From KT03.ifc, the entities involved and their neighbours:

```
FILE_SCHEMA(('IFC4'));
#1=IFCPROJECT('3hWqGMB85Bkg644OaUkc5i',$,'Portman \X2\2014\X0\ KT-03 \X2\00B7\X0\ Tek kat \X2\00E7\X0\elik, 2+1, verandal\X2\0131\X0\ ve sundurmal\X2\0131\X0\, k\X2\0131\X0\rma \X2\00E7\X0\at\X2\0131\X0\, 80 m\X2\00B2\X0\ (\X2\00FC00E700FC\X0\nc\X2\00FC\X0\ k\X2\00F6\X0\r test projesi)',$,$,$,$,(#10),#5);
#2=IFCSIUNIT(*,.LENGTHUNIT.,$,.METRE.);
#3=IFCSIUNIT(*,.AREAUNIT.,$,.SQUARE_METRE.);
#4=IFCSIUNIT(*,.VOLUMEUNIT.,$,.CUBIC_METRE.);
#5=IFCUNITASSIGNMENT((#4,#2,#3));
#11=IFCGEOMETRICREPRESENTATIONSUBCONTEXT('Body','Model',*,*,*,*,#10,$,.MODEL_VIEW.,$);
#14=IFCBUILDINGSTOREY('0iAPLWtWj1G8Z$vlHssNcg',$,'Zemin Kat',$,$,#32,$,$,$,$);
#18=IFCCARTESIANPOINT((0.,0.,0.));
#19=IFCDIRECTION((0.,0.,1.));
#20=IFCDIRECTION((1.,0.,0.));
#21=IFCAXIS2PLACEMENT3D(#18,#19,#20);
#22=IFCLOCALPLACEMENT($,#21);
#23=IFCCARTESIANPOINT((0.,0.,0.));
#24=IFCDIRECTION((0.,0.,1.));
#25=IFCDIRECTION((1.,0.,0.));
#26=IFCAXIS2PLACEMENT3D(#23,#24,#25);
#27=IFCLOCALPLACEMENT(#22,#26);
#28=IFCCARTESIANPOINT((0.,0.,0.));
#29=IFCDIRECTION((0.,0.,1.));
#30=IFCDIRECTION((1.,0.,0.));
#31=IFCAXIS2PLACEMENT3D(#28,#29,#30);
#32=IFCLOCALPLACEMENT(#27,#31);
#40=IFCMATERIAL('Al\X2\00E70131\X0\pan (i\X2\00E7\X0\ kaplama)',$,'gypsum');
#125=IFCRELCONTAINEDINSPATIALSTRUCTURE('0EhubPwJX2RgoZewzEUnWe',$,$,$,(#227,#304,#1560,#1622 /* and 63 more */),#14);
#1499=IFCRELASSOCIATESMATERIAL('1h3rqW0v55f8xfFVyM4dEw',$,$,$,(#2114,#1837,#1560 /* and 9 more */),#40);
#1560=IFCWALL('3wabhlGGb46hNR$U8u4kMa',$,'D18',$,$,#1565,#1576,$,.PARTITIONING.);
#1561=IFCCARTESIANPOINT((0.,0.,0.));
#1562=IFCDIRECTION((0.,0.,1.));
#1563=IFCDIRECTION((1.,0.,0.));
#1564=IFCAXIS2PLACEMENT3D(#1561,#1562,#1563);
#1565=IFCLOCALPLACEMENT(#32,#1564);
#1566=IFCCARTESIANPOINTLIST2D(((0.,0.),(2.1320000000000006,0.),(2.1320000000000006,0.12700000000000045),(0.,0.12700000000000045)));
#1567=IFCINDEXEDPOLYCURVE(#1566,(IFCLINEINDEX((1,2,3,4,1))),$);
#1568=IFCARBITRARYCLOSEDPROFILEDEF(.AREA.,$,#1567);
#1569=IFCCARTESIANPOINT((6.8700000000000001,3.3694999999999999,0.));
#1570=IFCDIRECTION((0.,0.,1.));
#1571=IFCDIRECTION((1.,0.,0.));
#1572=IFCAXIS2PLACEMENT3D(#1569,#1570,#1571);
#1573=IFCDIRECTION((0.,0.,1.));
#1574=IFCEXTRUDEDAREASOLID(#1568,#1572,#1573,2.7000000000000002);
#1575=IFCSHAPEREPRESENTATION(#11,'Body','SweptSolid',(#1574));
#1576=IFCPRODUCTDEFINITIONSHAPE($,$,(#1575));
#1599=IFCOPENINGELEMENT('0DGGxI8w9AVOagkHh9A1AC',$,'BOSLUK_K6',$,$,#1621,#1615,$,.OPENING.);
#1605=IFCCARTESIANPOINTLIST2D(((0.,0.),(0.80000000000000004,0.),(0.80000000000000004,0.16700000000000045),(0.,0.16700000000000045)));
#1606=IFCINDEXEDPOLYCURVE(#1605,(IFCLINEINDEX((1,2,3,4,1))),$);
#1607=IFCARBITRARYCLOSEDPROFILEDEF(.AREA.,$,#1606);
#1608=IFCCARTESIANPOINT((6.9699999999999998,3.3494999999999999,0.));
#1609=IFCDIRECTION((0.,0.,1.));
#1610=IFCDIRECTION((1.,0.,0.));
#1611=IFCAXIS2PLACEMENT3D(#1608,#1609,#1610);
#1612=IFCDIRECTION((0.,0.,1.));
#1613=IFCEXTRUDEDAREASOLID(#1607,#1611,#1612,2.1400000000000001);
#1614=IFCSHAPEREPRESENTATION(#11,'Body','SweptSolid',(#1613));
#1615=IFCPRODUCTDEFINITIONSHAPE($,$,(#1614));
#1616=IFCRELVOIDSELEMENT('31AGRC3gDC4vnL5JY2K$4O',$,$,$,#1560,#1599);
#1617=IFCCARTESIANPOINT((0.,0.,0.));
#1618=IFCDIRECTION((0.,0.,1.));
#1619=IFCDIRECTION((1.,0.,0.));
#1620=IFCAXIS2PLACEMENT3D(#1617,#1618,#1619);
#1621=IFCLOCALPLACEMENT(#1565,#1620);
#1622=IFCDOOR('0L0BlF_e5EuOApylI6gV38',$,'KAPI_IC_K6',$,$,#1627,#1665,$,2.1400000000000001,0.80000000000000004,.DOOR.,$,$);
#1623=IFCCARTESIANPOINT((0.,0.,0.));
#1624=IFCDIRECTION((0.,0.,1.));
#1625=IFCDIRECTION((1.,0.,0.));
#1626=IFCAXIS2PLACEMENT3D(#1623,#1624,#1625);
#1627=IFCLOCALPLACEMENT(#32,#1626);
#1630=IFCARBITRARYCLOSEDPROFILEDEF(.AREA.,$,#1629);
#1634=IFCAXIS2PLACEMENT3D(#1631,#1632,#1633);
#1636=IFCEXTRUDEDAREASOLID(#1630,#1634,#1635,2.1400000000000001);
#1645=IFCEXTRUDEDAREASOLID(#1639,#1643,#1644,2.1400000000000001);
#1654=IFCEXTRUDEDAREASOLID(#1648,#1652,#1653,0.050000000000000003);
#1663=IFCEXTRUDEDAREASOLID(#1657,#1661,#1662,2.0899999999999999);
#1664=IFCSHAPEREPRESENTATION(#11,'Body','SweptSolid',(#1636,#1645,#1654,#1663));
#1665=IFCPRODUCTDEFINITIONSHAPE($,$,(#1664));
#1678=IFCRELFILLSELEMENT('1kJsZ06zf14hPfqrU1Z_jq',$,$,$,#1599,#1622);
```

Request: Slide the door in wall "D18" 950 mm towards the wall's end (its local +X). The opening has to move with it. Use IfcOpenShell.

```python
import ifcopenshell
import ifcopenshell.api.geometry
import ifcopenshell.util.placement
import ifcopenshell.util.unit

model = ifcopenshell.open("KT03.ifc")
unit_scale = ifcopenshell.util.unit.calculate_unit_scale(model)

door = model.by_guid("0L0BlF_e5EuOApylI6gV38")
opening = door.FillsVoids[0].RelatingOpeningElement
wall = opening.VoidsElements[0].RelatingBuildingElement

wall_matrix = ifcopenshell.util.placement.get_local_placement(wall.ObjectPlacement)
shift = wall_matrix[:3, 0] * 0.95 / unit_scale
before = ifcopenshell.util.placement.get_local_placement(door.ObjectPlacement)[:3, 3].copy()

# The door is not placed relative to its opening, so move both.
for product in (opening, door):
    matrix = ifcopenshell.util.placement.get_local_placement(product.ObjectPlacement)
    matrix[:3, 3] += shift
    ifcopenshell.api.geometry.edit_object_placement(model, product=product, matrix=matrix, is_si=False)

after = ifcopenshell.util.placement.get_local_placement(door.ObjectPlacement)[:3, 3]
print("door moved by", (after - before).round(3) + 0.0)

model.write("KT03_rev.ifc")
```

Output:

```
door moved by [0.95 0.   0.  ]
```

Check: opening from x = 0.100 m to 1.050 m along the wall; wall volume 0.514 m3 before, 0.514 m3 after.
